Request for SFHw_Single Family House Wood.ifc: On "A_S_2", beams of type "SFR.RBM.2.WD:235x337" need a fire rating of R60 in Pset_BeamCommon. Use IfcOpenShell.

First a look at what the model holds.

```python
import ifcopenshell
import ifcopenshell.util.element

model = ifcopenshell.open("SFHw_Single Family House Wood.ifc")
print(model.schema)
storey = next(s for s in model.by_type("IfcBuildingStorey") if s.Name == "A_S_2")
beams = [e for e in ifcopenshell.util.element.get_decomposition(storey) if e.is_a("IfcBeam")]
seen = {}
for e in beams:
    element_type = ifcopenshell.util.element.get_type(e)
    key = (element_type.Name if element_type != e and element_type else None, ifcopenshell.util.element.get_pset(e, "Pset_BeamCommon", "FireRating"))
    seen[key] = seen.get(key, 0) + 1
for (name, value), count in sorted(seen.items(), key=str):
    print(count, "x", name, "|", value)
```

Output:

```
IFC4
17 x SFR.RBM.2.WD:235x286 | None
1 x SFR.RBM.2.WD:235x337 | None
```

```python
import ifcopenshell
import ifcopenshell.api.pset
import ifcopenshell.util.element

model = ifcopenshell.open("SFHw_Single Family House Wood.ifc")

storey = next(s for s in model.by_type("IfcBuildingStorey") if s.Name == "A_S_2")
beams = [e for e in ifcopenshell.util.element.get_decomposition(storey) if e.is_a("IfcBeam")]

count = 0
for e in beams:
    element_type = ifcopenshell.util.element.get_type(e)
    if element_type in (None, e) or element_type.Name != "SFR.RBM.2.WD:235x337":
        continue
    # add_pset returns the element's existing set when there is one.
    pset = ifcopenshell.api.pset.add_pset(model, product=e, name="Pset_BeamCommon")
    ifcopenshell.api.pset.edit_pset(model, pset=pset, properties={"FireRating": "R60"})
    count += 1

print(count, "beams updated")

model.write("SFHw_Single Family House Wood_edited.ifc")
```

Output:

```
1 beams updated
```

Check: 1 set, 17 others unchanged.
